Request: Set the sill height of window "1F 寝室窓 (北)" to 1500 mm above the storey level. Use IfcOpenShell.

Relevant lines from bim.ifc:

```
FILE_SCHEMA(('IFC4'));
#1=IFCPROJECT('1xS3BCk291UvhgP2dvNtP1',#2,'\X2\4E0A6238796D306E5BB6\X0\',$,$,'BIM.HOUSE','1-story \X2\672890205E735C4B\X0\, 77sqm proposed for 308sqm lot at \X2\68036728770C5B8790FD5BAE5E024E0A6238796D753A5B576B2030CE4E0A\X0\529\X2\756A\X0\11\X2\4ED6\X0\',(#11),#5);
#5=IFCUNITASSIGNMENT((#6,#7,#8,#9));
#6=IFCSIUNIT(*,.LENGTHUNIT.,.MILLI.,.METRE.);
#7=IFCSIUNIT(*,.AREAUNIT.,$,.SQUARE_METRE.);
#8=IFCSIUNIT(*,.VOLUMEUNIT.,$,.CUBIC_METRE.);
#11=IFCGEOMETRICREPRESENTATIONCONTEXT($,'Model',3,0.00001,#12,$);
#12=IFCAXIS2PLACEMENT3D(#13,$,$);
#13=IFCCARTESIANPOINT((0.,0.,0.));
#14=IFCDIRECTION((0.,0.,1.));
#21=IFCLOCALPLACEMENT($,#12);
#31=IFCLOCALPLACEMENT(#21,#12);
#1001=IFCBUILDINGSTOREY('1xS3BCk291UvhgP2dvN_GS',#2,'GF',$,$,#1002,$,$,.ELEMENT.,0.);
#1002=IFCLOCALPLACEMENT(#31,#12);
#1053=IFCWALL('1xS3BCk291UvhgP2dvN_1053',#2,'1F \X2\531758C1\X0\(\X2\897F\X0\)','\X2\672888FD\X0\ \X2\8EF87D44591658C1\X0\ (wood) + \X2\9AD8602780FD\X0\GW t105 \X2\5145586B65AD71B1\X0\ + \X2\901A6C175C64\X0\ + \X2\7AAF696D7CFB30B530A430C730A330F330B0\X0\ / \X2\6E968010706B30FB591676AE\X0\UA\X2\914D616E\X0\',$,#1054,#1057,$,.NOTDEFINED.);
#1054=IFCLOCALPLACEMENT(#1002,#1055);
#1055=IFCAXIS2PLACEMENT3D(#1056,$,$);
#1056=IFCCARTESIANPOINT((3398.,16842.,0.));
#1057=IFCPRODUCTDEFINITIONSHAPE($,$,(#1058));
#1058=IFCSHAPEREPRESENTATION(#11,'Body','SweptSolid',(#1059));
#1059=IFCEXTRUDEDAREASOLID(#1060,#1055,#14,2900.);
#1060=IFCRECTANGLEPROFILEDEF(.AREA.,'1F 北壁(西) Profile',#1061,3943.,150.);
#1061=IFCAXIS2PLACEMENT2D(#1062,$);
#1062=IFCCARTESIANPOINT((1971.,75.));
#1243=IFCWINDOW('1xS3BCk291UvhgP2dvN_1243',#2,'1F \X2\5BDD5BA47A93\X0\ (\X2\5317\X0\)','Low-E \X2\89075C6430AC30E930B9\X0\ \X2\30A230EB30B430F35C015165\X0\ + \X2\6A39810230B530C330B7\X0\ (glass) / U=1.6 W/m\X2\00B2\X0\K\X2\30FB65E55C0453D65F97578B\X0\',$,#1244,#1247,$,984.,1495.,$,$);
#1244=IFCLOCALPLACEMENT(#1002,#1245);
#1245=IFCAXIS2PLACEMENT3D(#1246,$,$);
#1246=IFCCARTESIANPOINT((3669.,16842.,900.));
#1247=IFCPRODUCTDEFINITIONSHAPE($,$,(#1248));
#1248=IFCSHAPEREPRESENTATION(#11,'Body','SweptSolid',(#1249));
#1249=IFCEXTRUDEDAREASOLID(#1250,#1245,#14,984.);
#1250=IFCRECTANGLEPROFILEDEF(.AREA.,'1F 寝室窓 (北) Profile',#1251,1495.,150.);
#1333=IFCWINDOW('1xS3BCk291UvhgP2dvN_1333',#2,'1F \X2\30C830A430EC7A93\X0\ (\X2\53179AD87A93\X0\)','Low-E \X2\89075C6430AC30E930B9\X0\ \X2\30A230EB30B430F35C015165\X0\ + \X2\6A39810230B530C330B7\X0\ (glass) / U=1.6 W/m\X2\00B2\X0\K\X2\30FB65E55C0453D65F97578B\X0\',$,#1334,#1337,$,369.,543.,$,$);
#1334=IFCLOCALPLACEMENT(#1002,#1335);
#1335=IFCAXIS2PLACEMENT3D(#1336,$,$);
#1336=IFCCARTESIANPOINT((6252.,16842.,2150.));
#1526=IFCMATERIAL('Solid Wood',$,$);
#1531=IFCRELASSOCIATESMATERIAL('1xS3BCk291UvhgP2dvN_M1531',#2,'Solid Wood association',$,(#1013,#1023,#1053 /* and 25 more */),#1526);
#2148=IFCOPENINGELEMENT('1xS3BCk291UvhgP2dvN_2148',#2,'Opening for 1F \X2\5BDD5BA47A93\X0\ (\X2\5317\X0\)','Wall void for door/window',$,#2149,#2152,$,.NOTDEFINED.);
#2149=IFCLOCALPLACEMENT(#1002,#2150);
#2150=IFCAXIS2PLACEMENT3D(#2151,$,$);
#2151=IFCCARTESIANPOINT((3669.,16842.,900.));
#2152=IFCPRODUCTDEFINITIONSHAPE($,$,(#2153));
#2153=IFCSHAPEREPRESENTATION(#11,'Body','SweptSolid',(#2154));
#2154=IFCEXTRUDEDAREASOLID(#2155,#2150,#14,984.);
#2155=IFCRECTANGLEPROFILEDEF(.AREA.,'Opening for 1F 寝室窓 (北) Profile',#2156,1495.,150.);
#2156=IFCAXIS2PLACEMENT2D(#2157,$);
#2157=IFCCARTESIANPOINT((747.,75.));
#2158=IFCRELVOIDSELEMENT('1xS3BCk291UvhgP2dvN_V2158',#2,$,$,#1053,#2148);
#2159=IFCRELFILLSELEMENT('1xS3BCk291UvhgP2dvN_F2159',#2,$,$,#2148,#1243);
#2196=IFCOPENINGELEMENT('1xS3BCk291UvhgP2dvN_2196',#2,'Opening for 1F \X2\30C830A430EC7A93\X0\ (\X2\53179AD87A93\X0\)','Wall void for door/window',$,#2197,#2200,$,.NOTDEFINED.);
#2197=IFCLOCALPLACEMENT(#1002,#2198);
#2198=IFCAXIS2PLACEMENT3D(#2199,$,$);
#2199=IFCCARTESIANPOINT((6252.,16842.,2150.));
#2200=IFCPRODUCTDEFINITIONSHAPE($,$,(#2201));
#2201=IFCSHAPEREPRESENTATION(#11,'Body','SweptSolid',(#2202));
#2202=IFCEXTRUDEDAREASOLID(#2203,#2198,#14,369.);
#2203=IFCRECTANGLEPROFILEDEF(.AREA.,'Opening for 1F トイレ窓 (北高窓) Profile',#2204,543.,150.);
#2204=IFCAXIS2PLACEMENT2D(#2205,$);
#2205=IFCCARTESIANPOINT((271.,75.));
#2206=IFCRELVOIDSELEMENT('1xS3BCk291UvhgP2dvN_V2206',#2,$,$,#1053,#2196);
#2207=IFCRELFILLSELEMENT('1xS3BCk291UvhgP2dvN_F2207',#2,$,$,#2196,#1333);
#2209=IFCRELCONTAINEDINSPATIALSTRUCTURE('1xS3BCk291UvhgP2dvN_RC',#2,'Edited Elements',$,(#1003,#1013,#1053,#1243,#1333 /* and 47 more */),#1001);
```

```python
import numpy as np
import ifcopenshell
import ifcopenshell.api.geometry
import ifcopenshell.geom
import ifcopenshell.util.element
import ifcopenshell.util.placement
import ifcopenshell.util.shape
import ifcopenshell.util.unit

model = ifcopenshell.open("bim.ifc")
unit_scale = ifcopenshell.util.unit.calculate_unit_scale(model)

window = model.by_guid("1xS3BCk291UvhgP2dvN_1243")
opening = window.FillsVoids[0].RelatingOpeningElement
storey = ifcopenshell.util.element.get_container(window, ifc_class="IfcBuildingStorey")
level = ifcopenshell.util.placement.get_local_placement(storey.ObjectPlacement)[2, 3]

# The opening's origin need not be at the sill, so measure its lowest point.
shape = ifcopenshell.geom.create_shape(ifcopenshell.geom.settings(), opening)
bottom = ifcopenshell.util.shape.get_shape_bottom_elevation(shape, shape.geometry) / unit_scale
dz = level + 1.5 / unit_scale - bottom

shift = np.array([0.0, 0.0, dz])
# The window is not placed relative to its opening, so move both.
for product in (opening, window):
    matrix = ifcopenshell.util.placement.get_local_placement(product.ObjectPlacement)
    matrix[:3, 3] += shift
    ifcopenshell.api.geometry.edit_object_placement(model, product=product, matrix=matrix, is_si=False)

print(f"moved by {dz * unit_scale:+.3f} m")

model.write("bim_updated.ifc")
```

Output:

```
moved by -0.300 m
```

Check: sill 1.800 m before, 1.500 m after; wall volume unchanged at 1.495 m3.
